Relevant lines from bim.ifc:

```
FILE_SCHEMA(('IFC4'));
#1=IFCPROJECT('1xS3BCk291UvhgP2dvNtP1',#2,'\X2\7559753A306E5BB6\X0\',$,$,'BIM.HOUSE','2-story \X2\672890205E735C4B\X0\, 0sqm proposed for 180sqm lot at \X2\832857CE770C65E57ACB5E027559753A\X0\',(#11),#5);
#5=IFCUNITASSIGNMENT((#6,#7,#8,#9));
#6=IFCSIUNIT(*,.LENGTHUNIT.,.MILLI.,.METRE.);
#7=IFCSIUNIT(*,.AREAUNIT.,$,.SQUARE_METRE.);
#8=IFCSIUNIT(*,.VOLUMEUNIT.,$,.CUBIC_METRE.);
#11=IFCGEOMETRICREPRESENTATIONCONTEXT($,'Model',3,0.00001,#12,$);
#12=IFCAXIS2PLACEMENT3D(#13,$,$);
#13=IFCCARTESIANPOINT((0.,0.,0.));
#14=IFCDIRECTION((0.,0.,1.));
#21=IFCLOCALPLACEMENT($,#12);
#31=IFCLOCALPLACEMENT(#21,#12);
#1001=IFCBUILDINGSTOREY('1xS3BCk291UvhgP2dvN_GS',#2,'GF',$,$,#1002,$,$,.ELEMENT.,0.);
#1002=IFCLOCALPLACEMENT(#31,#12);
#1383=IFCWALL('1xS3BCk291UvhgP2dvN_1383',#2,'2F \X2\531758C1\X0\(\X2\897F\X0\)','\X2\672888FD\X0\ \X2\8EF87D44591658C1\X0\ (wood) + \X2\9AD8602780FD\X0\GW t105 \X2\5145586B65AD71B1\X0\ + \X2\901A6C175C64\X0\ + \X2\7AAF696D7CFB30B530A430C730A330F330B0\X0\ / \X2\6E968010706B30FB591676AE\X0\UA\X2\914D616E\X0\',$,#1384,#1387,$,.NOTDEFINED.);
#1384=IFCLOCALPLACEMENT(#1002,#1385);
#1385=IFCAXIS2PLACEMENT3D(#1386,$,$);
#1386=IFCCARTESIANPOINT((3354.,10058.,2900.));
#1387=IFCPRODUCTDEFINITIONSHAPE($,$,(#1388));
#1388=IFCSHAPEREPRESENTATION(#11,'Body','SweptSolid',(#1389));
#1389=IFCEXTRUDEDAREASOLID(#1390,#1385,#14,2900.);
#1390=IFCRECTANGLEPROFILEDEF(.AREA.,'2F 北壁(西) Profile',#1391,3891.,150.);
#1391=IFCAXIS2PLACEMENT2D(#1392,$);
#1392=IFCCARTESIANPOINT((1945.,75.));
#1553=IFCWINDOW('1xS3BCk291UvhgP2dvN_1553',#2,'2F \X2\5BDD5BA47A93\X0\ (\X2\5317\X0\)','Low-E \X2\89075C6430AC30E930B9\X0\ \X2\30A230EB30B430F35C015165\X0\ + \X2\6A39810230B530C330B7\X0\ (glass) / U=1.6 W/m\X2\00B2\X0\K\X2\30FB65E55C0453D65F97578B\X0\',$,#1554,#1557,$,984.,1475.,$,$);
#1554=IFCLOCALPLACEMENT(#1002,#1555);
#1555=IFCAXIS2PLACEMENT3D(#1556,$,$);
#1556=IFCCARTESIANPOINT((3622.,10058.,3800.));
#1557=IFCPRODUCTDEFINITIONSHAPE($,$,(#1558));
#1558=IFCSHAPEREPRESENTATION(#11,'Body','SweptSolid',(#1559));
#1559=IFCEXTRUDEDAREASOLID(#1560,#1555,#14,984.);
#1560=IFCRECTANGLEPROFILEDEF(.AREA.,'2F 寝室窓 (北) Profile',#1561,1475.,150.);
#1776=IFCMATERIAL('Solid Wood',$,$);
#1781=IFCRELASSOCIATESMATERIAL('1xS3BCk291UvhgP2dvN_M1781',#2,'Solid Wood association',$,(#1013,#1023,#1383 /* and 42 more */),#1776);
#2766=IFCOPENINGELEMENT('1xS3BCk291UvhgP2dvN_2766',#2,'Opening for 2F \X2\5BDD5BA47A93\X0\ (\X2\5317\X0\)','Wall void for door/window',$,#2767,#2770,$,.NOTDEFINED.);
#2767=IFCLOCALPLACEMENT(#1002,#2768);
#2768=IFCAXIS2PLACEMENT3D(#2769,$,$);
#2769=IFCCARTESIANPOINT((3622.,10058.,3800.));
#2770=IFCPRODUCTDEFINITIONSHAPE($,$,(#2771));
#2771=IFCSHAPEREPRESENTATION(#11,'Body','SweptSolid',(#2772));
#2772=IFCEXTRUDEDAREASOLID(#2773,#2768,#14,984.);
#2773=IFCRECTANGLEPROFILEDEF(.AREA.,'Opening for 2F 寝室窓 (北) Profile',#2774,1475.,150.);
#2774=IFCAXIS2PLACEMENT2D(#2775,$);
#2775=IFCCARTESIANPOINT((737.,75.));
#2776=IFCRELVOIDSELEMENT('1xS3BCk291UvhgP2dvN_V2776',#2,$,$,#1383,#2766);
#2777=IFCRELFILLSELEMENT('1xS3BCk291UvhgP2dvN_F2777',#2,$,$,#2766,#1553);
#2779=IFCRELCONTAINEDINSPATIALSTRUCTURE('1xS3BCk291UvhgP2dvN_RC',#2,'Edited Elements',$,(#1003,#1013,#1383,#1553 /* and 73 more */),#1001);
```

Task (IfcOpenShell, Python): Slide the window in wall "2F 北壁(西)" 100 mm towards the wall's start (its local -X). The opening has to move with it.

```python
import ifcopenshell
import ifcopenshell.api.geometry
import ifcopenshell.util.placement
import ifcopenshell.util.unit

model = ifcopenshell.open("bim.ifc")
unit_scale = ifcopenshell.util.unit.calculate_unit_scale(model)

window = model.by_guid("1xS3BCk291UvhgP2dvN_1553")
opening = window.FillsVoids[0].RelatingOpeningElement
wall = opening.VoidsElements[0].RelatingBuildingElement

wall_matrix = ifcopenshell.util.placement.get_local_placement(wall.ObjectPlacement)
shift = wall_matrix[:3, 0] * -0.1 / unit_scale
before = ifcopenshell.util.placement.get_local_placement(window.ObjectPlacement)[:3, 3].copy()

# The window is not placed relative to its opening, so move both.
for product in (opening, window):
    matrix = ifcopenshell.util.placement.get_local_placement(product.ObjectPlacement)
    matrix[:3, 3] += shift
    ifcopenshell.api.geometry.edit_object_placement(model, product=product, matrix=matrix, is_si=False)

after = ifcopenshell.util.placement.get_local_placement(window.ObjectPlacement)[:3, 3]
print("window moved by", (after - before).round(3) + 0.0)

model.write("bim_updated.ifc")
```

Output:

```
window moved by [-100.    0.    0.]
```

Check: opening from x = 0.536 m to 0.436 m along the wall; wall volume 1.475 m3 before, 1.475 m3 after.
